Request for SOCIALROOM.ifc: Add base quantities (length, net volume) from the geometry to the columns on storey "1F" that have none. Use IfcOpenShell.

First a look at what the model holds.

```python
import ifcopenshell
import ifcopenshell.util.element
import ifcopenshell.util.unit

model = ifcopenshell.open("SOCIALROOM.ifc")
print(model.schema)
for unit_type in ("LENGTHUNIT", "AREAUNIT", "VOLUMEUNIT"):
    print(unit_type, ifcopenshell.util.unit.calculate_unit_scale(model, unit_type))
storey = next(s for s in model.by_type("IfcBuildingStorey") if s.Name == "1F")
columns = [e for e in ifcopenshell.util.element.get_decomposition(storey) if e.is_a("IfcColumn")]
for e in sorted(columns, key=lambda e: e.id()):
    print(e.id(), e.is_a(), e.Name, list(ifcopenshell.util.element.get_psets(e, qtos_only=True)), sep=" | ")
```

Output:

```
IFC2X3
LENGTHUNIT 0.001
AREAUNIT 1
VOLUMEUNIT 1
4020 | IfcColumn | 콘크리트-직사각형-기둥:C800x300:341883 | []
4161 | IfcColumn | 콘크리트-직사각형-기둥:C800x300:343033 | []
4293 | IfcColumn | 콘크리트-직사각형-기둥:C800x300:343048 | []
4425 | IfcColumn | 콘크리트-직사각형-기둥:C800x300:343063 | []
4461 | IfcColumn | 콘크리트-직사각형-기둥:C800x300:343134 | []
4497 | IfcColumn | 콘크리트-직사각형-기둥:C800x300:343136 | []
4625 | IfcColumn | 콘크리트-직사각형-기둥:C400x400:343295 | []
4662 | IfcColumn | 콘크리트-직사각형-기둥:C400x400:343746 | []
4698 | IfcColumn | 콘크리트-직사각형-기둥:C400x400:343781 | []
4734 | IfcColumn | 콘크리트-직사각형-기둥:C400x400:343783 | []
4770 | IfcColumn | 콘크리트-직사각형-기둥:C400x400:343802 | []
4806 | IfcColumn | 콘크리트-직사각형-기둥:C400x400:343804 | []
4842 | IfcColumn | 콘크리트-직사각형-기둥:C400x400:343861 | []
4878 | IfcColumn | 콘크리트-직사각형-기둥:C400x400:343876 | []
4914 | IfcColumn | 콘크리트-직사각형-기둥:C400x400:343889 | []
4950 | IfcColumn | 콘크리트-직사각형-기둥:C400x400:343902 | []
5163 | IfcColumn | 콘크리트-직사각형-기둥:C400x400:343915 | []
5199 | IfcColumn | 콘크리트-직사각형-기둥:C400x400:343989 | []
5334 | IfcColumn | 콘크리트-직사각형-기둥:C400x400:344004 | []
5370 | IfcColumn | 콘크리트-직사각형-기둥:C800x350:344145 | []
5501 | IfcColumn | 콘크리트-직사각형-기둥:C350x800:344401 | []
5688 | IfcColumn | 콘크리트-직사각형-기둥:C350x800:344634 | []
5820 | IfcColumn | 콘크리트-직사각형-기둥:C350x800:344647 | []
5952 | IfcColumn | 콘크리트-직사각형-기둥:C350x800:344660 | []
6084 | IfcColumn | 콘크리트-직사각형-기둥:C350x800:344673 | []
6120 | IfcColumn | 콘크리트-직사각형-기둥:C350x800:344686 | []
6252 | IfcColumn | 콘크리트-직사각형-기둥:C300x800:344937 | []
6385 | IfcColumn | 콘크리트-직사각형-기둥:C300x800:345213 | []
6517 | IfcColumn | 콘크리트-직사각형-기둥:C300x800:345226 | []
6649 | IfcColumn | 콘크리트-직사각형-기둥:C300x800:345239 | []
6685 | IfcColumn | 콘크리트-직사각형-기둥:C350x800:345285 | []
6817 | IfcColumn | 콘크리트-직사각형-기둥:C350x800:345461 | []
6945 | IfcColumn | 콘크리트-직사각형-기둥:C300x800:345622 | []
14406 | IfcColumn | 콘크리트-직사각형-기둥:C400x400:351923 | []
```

```python
import ifcopenshell
import ifcopenshell.api.pset
import ifcopenshell.geom
import ifcopenshell.util.element
import ifcopenshell.util.shape
import ifcopenshell.util.unit

model = ifcopenshell.open("SOCIALROOM.ifc")
unit_scale = ifcopenshell.util.unit.calculate_unit_scale(model)
volume_scale = ifcopenshell.util.unit.calculate_unit_scale(model, "VOLUMEUNIT")
settings = ifcopenshell.geom.settings()

storey = next(s for s in model.by_type("IfcBuildingStorey") if s.Name == "1F")
columns = [e for e in ifcopenshell.util.element.get_decomposition(storey) if e.is_a("IfcColumn")]

for e in sorted(columns, key=lambda e: e.id()):
    if ifcopenshell.util.element.get_psets(e, qtos_only=True, should_inherit=False):
        continue
    # Geometry comes back in metres, in the element's own axes.
    shape = ifcopenshell.geom.create_shape(settings, e)
    values = {
        "Length": ifcopenshell.util.shape.get_z(shape.geometry) / unit_scale,
        "NetVolume": ifcopenshell.util.shape.get_volume(shape.geometry) / volume_scale,
    }
    qto = ifcopenshell.api.pset.add_qto(model, product=e, name="BaseQuantities")
    ifcopenshell.api.pset.edit_qto(model, qto=qto, properties=values)
    print(e.id(), {k: round(v, 3) for k, v in values.items()})

model.write("SOCIALROOM_updated.ifc")
```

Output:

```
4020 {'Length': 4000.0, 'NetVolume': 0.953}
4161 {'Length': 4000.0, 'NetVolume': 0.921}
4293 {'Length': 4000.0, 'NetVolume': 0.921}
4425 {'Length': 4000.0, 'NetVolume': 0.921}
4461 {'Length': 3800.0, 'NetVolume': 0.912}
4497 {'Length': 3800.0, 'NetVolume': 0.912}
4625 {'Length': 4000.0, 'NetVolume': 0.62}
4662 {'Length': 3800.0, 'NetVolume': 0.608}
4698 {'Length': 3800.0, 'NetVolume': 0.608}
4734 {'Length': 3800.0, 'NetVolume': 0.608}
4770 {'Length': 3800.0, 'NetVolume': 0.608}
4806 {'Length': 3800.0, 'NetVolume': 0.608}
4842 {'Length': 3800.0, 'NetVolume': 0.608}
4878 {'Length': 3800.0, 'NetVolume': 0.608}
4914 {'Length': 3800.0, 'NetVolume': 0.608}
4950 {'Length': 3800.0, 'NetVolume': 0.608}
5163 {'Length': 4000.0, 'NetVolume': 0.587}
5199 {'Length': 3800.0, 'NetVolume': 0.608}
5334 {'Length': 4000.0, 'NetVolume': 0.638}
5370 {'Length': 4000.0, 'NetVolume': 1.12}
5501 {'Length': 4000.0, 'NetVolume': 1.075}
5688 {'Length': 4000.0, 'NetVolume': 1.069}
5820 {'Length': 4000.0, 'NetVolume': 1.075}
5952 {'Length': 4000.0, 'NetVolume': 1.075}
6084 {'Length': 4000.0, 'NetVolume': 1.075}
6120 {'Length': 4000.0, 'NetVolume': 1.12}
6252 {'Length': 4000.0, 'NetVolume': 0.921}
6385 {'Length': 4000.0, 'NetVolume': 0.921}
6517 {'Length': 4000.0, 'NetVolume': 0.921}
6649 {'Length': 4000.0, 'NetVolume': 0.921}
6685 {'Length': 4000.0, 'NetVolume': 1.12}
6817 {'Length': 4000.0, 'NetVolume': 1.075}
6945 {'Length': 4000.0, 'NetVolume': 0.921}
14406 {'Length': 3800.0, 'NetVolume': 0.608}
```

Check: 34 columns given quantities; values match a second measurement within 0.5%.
